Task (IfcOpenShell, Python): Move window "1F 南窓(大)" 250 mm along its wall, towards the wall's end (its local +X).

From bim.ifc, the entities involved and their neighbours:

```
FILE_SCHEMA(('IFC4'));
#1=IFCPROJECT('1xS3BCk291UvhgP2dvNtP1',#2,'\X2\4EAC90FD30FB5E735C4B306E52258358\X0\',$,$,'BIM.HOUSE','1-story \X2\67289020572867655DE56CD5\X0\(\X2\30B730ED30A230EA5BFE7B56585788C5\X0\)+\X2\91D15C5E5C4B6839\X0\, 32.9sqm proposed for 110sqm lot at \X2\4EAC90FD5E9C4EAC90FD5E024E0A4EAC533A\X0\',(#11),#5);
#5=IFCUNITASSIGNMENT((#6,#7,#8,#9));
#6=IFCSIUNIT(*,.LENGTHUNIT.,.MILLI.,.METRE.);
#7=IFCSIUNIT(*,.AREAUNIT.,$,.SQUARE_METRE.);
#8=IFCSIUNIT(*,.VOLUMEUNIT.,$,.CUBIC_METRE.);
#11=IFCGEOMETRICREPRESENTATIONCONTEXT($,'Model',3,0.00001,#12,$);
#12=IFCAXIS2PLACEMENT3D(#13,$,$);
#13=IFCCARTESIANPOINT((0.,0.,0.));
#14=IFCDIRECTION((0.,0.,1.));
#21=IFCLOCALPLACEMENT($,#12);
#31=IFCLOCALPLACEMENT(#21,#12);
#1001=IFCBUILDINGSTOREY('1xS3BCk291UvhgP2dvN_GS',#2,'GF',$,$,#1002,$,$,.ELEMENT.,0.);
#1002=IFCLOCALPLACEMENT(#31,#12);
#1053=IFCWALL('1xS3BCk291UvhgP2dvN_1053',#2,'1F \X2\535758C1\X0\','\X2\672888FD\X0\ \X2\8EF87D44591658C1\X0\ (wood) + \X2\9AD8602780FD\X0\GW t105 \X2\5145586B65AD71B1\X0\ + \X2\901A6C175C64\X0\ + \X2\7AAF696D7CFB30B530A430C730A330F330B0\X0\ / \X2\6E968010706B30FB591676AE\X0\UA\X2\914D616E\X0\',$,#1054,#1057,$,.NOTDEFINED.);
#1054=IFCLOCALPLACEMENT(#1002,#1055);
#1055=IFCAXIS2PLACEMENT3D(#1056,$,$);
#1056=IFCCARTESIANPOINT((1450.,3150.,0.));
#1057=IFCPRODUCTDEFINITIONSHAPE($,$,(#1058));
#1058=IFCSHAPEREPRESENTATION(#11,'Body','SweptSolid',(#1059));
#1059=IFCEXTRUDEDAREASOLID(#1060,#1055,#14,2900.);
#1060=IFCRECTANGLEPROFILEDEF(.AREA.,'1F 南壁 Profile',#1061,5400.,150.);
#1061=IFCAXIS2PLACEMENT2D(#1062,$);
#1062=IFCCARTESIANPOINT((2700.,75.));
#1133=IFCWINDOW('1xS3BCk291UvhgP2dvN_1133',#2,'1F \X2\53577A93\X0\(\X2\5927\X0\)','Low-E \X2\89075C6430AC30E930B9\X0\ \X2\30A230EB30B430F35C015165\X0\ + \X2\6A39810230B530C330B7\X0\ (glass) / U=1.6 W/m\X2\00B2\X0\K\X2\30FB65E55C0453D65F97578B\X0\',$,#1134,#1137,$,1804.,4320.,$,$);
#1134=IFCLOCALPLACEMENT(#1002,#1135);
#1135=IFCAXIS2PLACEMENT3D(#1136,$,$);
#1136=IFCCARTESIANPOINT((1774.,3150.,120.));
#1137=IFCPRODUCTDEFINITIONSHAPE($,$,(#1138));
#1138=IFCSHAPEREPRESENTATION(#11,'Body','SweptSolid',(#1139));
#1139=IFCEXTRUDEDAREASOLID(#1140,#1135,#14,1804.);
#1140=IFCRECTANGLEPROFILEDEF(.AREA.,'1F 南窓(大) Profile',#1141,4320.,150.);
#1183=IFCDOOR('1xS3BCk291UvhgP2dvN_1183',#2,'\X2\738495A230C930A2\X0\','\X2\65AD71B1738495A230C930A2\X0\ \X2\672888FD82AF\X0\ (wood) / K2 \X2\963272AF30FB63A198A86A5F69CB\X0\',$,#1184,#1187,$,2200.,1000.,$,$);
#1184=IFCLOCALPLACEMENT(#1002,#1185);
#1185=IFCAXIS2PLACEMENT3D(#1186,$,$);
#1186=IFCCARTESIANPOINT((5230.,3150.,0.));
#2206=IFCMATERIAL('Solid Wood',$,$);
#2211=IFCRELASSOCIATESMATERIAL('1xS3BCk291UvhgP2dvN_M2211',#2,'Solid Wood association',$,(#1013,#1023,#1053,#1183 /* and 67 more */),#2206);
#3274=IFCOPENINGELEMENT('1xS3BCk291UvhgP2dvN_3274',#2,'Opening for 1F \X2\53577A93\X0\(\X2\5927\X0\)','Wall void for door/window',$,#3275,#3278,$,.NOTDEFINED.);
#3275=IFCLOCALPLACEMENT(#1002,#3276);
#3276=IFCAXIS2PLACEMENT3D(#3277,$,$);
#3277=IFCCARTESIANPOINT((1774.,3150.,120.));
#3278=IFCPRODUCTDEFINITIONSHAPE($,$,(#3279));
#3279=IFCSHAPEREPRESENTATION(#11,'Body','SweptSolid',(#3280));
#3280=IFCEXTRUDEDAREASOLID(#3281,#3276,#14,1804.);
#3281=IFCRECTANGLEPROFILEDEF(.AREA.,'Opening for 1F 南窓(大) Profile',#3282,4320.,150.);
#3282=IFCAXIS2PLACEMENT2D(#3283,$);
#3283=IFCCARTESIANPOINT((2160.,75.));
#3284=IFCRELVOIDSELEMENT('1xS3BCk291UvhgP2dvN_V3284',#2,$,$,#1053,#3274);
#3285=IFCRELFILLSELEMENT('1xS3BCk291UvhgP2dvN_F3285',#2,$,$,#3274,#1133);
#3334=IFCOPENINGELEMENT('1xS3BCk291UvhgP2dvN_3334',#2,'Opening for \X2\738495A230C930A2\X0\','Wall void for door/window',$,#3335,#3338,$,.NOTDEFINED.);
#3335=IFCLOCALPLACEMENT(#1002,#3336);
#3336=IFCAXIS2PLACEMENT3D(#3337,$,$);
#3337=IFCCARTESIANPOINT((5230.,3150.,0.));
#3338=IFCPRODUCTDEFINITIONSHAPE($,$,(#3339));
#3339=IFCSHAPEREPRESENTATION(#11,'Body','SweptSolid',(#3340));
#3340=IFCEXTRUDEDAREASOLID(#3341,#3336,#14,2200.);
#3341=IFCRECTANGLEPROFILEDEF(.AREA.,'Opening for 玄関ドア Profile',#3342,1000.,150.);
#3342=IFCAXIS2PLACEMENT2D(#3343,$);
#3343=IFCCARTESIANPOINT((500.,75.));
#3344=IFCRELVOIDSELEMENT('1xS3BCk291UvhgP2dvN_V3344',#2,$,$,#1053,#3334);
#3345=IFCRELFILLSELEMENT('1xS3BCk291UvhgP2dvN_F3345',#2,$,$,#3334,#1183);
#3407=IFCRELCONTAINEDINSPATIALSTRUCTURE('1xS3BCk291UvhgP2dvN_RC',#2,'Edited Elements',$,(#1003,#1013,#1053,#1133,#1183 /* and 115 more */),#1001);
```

```python
import ifcopenshell
import ifcopenshell.api.geometry
import ifcopenshell.util.placement
import ifcopenshell.util.unit

model = ifcopenshell.open("bim.ifc")
unit_scale = ifcopenshell.util.unit.calculate_unit_scale(model)

window = model.by_guid("1xS3BCk291UvhgP2dvN_1133")
opening = window.FillsVoids[0].RelatingOpeningElement
wall = opening.VoidsElements[0].RelatingBuildingElement

wall_matrix = ifcopenshell.util.placement.get_local_placement(wall.ObjectPlacement)
shift = wall_matrix[:3, 0] * 0.25 / unit_scale
before = ifcopenshell.util.placement.get_local_placement(window.ObjectPlacement)[:3, 3].copy()

# The window is not placed relative to its opening, so move both.
for product in (opening, window):
    matrix = ifcopenshell.util.placement.get_local_placement(product.ObjectPlacement)
    matrix[:3, 3] += shift
    ifcopenshell.api.geometry.edit_object_placement(model, product=product, matrix=matrix, is_si=False)

after = ifcopenshell.util.placement.get_local_placement(window.ObjectPlacement)[:3, 3]
print("window moved by", (after - before).round(3) + 0.0)

model.write("bim_v2.ifc")
```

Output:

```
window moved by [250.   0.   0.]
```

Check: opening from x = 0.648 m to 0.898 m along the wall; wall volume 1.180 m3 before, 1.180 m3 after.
